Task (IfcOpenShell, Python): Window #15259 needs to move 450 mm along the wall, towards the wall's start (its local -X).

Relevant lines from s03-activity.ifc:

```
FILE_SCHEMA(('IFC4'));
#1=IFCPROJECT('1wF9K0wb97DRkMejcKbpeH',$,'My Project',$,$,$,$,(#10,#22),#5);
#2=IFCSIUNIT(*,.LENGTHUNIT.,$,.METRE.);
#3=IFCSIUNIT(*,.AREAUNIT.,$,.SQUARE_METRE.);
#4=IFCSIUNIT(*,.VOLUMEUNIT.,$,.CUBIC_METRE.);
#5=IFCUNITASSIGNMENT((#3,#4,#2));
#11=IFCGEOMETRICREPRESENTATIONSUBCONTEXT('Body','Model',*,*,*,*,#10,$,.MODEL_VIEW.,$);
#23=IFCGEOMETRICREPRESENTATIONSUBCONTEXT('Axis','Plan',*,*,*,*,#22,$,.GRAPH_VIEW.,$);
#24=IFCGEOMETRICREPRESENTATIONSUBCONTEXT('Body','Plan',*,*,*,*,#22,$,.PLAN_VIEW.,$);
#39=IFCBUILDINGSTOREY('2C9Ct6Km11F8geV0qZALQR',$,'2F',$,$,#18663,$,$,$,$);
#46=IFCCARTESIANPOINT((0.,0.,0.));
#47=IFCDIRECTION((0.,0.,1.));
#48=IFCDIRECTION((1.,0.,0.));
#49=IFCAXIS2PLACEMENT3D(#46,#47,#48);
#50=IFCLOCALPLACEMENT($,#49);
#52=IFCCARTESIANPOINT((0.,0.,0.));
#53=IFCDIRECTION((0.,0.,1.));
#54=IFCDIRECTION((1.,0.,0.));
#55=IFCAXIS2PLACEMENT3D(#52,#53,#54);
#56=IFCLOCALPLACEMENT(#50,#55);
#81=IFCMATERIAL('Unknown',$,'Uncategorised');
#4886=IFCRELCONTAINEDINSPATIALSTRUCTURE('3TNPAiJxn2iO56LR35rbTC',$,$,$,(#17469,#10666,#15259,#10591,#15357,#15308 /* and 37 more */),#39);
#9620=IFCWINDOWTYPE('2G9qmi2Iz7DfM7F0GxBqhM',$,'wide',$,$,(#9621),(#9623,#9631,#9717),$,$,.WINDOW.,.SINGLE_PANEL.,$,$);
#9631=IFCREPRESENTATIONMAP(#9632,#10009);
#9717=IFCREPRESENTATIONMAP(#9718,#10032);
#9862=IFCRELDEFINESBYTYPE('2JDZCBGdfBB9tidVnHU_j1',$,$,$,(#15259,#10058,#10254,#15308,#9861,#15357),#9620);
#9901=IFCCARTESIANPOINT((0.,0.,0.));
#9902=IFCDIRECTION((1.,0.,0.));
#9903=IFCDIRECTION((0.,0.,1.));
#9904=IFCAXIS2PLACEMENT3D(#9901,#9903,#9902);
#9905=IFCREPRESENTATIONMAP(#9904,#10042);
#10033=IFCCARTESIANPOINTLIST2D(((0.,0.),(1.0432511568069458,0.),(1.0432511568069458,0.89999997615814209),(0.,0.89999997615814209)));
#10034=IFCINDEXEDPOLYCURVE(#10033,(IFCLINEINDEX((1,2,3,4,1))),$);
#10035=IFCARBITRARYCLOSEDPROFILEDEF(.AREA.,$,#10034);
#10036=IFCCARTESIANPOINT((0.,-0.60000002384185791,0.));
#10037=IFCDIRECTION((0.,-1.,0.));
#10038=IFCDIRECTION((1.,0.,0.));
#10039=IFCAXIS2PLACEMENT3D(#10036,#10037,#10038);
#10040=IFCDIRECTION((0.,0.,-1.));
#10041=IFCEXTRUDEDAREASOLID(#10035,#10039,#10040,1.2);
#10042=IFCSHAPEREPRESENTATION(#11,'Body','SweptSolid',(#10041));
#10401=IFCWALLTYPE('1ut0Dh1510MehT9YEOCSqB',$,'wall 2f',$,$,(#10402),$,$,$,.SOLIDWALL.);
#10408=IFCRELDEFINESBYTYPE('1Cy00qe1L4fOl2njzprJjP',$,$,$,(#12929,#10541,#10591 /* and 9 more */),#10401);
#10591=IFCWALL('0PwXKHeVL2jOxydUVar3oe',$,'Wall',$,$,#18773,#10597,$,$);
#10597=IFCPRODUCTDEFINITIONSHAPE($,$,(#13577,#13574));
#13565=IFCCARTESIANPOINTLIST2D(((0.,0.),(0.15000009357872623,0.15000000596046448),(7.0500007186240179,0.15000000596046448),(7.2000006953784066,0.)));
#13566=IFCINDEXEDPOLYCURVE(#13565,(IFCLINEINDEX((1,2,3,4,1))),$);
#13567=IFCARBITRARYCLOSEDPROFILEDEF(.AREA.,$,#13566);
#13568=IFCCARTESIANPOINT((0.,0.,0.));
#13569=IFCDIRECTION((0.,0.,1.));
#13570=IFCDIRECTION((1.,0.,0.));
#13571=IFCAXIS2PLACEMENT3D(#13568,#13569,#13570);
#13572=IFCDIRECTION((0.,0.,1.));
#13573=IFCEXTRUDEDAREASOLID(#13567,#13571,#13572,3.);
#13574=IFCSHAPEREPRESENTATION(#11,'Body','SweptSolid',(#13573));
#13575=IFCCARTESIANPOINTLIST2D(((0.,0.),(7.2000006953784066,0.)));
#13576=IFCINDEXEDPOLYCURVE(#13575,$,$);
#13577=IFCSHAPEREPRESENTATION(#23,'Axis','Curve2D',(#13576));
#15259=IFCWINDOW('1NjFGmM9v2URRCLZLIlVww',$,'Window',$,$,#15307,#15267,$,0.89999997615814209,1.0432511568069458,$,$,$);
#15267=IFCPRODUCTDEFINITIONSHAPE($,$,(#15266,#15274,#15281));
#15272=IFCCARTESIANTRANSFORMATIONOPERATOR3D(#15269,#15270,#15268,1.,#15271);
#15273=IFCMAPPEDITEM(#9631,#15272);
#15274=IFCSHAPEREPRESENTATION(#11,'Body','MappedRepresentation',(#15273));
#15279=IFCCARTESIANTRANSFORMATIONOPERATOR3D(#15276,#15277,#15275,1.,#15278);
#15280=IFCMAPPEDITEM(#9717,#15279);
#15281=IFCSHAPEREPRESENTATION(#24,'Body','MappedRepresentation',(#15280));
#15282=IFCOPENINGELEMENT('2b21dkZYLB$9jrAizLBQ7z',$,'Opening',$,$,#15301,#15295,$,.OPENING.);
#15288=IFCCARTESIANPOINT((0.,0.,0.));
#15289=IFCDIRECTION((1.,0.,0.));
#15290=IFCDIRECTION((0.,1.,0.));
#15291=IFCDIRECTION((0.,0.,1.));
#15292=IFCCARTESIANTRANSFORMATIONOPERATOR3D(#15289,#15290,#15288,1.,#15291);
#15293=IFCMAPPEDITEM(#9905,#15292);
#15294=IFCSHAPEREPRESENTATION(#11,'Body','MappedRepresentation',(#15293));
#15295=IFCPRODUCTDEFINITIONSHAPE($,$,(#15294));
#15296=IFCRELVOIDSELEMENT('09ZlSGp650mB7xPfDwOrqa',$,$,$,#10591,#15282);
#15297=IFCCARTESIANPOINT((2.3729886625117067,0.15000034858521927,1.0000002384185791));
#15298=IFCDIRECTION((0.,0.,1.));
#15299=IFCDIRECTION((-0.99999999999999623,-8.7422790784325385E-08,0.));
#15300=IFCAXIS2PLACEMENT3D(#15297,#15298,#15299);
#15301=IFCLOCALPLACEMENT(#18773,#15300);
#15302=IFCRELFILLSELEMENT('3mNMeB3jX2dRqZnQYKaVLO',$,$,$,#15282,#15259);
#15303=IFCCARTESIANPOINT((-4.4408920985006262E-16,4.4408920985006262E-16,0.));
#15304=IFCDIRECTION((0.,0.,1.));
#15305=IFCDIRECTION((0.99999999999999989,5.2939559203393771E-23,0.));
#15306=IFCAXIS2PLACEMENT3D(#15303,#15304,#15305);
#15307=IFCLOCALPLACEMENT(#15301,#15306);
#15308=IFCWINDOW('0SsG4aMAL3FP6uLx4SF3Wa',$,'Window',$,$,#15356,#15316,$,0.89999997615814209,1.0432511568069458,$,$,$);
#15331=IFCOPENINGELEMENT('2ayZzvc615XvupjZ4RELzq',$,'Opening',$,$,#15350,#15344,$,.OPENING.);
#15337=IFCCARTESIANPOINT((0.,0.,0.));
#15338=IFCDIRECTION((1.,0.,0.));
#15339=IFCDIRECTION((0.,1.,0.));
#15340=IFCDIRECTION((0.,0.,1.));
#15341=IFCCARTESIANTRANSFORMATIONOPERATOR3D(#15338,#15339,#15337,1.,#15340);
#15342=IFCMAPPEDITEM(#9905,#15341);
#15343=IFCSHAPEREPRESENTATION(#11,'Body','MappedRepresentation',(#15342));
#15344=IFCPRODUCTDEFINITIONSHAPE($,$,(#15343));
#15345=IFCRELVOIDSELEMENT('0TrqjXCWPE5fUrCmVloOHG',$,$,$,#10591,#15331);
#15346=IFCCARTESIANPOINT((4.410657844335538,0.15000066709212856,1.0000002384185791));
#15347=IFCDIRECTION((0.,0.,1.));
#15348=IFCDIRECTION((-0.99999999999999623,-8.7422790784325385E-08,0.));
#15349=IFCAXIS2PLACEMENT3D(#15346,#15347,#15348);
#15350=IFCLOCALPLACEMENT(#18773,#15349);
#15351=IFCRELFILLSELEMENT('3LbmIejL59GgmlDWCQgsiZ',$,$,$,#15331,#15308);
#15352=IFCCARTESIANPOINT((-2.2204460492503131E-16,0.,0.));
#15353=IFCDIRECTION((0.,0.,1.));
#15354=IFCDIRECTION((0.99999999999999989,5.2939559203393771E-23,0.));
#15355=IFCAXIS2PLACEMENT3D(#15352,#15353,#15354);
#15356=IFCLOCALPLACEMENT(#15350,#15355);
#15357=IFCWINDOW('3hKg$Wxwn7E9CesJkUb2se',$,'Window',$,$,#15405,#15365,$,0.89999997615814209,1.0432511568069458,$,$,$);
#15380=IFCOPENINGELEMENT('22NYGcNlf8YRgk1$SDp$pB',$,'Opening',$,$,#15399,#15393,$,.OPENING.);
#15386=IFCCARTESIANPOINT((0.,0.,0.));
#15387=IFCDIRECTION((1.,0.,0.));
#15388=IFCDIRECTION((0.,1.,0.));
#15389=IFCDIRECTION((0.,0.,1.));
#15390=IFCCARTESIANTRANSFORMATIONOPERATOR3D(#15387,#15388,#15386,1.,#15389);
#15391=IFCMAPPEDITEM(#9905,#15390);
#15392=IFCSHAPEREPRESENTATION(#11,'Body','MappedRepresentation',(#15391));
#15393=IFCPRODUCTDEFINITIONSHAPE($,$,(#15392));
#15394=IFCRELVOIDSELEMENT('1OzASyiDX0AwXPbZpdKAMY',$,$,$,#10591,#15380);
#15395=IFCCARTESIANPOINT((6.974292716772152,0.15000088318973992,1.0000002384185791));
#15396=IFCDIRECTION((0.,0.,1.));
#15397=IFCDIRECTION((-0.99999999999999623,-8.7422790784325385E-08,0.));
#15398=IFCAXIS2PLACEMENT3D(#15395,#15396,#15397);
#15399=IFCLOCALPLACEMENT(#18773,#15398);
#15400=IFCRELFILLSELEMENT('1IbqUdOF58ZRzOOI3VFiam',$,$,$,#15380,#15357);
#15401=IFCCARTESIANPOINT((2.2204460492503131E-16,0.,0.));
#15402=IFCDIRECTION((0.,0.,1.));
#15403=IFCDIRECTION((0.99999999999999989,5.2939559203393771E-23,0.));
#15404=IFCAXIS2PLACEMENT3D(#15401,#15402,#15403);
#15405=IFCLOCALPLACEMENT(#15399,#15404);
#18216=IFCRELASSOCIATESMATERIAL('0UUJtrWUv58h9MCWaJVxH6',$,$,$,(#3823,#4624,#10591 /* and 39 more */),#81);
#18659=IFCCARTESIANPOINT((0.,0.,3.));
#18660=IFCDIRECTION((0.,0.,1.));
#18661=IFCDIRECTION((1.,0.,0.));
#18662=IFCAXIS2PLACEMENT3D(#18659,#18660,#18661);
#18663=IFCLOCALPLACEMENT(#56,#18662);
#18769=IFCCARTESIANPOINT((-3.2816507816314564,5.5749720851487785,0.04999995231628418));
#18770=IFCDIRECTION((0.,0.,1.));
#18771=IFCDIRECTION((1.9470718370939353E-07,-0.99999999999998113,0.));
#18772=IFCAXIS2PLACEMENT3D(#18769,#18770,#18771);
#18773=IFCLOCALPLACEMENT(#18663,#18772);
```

```python
import ifcopenshell
import ifcopenshell.api.geometry
import ifcopenshell.util.placement

model = ifcopenshell.open("s03-activity.ifc")

window = model.by_id(15259)
opening = window.FillsVoids[0].RelatingOpeningElement
wall = opening.VoidsElements[0].RelatingBuildingElement

wall_matrix = ifcopenshell.util.placement.get_local_placement(wall.ObjectPlacement)
shift = wall_matrix[:3, 0] * -0.45
before = ifcopenshell.util.placement.get_local_placement(window.ObjectPlacement)[:3, 3].copy()

# The window is placed relative to its opening, so it follows when the opening moves.
matrix = ifcopenshell.util.placement.get_local_placement(opening.ObjectPlacement)
matrix[:3, 3] += shift
ifcopenshell.api.geometry.edit_object_placement(
    model, product=opening, matrix=matrix, is_si=False, should_transform_children=True
)

after = ifcopenshell.util.placement.get_local_placement(window.ObjectPlacement)[:3, 3]
print("window moved by", (after - before).round(3) + 0.0)

model.write("s03-activity-out.ifc")
```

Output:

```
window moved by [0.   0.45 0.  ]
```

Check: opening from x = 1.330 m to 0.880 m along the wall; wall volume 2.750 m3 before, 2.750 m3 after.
